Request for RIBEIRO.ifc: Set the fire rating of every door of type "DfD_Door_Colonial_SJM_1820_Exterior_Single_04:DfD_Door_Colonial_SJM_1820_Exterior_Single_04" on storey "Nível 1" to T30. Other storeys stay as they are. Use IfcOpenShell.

First a look at what the model holds.

```python
import ifcopenshell
import ifcopenshell.util.element

model = ifcopenshell.open("RIBEIRO.ifc")
print(model.schema)
storey = next(s for s in model.by_type("IfcBuildingStorey") if s.Name == "Nível 1")
doors = [e for e in ifcopenshell.util.element.get_decomposition(storey) if e.is_a("IfcDoor")]
seen = {}
for e in doors:
    element_type = ifcopenshell.util.element.get_type(e)
    key = (element_type.Name if element_type != e and element_type else None, ifcopenshell.util.element.get_pset(e, "Pset_DoorCommon", "FireRating"))
    seen[key] = seen.get(key, 0) + 1
for (name, value), count in sorted(seen.items(), key=str):
    print(count, "x", name, "|", value)
```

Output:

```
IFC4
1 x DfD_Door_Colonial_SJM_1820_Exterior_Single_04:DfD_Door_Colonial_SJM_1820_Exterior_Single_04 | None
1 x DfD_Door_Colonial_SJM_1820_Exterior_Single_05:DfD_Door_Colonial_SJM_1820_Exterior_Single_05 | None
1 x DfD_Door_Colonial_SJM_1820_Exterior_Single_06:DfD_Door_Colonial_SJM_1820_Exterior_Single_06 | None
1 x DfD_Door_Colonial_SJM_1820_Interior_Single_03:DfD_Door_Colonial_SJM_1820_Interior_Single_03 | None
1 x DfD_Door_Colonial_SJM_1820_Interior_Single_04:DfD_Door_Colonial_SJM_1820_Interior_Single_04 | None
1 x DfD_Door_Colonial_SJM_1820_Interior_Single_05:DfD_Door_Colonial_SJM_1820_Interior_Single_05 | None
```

```python
import ifcopenshell
import ifcopenshell.api.pset
import ifcopenshell.util.element

model = ifcopenshell.open("RIBEIRO.ifc")

storey = next(s for s in model.by_type("IfcBuildingStorey") if s.Name == "Nível 1")
doors = [e for e in ifcopenshell.util.element.get_decomposition(storey) if e.is_a("IfcDoor")]

count = 0
for e in doors:
    element_type = ifcopenshell.util.element.get_type(e)
    if element_type in (None, e) or element_type.Name != "DfD_Door_Colonial_SJM_1820_Exterior_Single_04:DfD_Door_Colonial_SJM_1820_Exterior_Single_04":
        continue
    # add_pset returns the element's existing set when there is one.
    pset = ifcopenshell.api.pset.add_pset(model, product=e, name="Pset_DoorCommon")
    ifcopenshell.api.pset.edit_pset(model, pset=pset, properties={"FireRating": "T30"})
    count += 1

print(count, "doors updated")

model.write("RIBEIRO-out.ifc")
```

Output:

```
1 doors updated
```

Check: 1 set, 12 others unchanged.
